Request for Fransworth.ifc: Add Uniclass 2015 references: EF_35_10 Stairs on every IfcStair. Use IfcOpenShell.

First a look at what the model holds.

```python
import ifcopenshell

model = ifcopenshell.open("Fransworth.ifc")
print(model.schema)
print("classifications:", [c.Name for c in model.by_type("IfcClassification")])
for ifc_class in ("IfcDoor", "IfcRoof", "IfcStair", "IfcWall", "IfcWindow"):
    print(ifc_class, len(model.by_type(ifc_class)))
```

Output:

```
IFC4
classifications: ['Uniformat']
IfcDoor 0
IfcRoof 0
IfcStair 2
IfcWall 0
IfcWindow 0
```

```python
import ifcopenshell
import ifcopenshell.api.classification

model = ifcopenshell.open("Fransworth.ifc")

system = ifcopenshell.api.classification.add_classification(model, classification="Uniclass 2015")

codes = {
    "IfcStair": ("EF_35_10", "Stairs"),
}
for ifc_class, (code, name) in codes.items():
    products = model.by_type(ifc_class)
    ifcopenshell.api.classification.add_reference(
        model, products=products, classification=system, identification=code, name=name
    )
    print(code, len(products))

model.write("Fransworth-out.ifc")
```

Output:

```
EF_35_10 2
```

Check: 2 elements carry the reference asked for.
